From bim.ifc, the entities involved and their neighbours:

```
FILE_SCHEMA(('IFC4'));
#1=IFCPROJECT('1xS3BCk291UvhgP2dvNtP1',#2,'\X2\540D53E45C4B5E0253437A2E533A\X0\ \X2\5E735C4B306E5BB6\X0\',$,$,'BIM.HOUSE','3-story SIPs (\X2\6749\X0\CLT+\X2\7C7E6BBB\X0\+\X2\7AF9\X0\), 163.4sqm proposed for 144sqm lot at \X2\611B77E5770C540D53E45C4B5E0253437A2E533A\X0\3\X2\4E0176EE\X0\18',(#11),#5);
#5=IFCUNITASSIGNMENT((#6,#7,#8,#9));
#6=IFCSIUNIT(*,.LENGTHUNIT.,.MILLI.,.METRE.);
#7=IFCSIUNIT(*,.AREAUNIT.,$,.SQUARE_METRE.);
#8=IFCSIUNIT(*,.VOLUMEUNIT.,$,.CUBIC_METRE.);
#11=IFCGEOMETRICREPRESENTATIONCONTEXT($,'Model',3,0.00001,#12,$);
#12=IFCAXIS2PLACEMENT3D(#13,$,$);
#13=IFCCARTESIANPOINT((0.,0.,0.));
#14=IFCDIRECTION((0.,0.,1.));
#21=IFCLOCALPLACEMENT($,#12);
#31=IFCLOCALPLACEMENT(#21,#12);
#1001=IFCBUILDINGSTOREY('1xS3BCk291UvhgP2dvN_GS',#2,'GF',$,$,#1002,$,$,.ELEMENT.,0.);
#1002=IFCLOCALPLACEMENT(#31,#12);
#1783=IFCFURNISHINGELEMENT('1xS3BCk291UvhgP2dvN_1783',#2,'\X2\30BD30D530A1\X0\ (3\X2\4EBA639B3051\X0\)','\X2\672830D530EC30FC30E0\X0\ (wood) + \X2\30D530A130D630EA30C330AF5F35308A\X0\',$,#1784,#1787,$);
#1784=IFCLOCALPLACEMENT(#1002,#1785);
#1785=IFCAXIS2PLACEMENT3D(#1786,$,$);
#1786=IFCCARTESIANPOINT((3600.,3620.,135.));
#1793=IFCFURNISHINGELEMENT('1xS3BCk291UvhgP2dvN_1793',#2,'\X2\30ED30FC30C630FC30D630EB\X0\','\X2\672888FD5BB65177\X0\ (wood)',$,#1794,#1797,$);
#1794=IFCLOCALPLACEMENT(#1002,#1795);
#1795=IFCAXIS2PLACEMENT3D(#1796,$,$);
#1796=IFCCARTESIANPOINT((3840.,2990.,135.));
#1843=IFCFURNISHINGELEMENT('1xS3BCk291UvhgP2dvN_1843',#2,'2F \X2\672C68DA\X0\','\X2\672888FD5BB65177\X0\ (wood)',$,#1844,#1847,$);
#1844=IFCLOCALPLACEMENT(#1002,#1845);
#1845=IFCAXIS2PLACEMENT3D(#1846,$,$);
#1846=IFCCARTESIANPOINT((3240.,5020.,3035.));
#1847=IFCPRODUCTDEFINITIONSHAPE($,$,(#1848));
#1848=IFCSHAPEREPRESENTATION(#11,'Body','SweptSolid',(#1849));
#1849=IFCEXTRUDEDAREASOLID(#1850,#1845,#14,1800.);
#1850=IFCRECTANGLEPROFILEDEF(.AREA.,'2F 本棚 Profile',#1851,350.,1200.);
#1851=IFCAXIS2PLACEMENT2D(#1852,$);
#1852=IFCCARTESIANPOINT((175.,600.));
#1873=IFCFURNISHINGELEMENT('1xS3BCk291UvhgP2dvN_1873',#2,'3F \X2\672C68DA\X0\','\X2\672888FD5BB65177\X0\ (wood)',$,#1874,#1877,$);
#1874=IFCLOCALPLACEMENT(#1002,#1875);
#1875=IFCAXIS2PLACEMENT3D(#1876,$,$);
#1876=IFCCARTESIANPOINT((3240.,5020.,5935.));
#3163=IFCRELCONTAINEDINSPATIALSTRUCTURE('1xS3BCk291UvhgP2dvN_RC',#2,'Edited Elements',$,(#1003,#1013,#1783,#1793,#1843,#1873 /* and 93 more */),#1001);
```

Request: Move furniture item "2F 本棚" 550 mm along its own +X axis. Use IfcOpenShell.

```python
import ifcopenshell
import ifcopenshell.api.geometry
import ifcopenshell.util.placement

model = ifcopenshell.open("bim.ifc")

item = model.by_guid("1xS3BCk291UvhgP2dvN_1843")
matrix = ifcopenshell.util.placement.get_local_placement(item.ObjectPlacement)
matrix[:3, 3] += matrix[:3, 0] * 550.0
ifcopenshell.api.geometry.edit_object_placement(model, product=item, matrix=matrix, is_si=False)

print(ifcopenshell.util.placement.get_local_placement(item.ObjectPlacement).round(3) + 0.0)

model.write("bim_updated.ifc")
```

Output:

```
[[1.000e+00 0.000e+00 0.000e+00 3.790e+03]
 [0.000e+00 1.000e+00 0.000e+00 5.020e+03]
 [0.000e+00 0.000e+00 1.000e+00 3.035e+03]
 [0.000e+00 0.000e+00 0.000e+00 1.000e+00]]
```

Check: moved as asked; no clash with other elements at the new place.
